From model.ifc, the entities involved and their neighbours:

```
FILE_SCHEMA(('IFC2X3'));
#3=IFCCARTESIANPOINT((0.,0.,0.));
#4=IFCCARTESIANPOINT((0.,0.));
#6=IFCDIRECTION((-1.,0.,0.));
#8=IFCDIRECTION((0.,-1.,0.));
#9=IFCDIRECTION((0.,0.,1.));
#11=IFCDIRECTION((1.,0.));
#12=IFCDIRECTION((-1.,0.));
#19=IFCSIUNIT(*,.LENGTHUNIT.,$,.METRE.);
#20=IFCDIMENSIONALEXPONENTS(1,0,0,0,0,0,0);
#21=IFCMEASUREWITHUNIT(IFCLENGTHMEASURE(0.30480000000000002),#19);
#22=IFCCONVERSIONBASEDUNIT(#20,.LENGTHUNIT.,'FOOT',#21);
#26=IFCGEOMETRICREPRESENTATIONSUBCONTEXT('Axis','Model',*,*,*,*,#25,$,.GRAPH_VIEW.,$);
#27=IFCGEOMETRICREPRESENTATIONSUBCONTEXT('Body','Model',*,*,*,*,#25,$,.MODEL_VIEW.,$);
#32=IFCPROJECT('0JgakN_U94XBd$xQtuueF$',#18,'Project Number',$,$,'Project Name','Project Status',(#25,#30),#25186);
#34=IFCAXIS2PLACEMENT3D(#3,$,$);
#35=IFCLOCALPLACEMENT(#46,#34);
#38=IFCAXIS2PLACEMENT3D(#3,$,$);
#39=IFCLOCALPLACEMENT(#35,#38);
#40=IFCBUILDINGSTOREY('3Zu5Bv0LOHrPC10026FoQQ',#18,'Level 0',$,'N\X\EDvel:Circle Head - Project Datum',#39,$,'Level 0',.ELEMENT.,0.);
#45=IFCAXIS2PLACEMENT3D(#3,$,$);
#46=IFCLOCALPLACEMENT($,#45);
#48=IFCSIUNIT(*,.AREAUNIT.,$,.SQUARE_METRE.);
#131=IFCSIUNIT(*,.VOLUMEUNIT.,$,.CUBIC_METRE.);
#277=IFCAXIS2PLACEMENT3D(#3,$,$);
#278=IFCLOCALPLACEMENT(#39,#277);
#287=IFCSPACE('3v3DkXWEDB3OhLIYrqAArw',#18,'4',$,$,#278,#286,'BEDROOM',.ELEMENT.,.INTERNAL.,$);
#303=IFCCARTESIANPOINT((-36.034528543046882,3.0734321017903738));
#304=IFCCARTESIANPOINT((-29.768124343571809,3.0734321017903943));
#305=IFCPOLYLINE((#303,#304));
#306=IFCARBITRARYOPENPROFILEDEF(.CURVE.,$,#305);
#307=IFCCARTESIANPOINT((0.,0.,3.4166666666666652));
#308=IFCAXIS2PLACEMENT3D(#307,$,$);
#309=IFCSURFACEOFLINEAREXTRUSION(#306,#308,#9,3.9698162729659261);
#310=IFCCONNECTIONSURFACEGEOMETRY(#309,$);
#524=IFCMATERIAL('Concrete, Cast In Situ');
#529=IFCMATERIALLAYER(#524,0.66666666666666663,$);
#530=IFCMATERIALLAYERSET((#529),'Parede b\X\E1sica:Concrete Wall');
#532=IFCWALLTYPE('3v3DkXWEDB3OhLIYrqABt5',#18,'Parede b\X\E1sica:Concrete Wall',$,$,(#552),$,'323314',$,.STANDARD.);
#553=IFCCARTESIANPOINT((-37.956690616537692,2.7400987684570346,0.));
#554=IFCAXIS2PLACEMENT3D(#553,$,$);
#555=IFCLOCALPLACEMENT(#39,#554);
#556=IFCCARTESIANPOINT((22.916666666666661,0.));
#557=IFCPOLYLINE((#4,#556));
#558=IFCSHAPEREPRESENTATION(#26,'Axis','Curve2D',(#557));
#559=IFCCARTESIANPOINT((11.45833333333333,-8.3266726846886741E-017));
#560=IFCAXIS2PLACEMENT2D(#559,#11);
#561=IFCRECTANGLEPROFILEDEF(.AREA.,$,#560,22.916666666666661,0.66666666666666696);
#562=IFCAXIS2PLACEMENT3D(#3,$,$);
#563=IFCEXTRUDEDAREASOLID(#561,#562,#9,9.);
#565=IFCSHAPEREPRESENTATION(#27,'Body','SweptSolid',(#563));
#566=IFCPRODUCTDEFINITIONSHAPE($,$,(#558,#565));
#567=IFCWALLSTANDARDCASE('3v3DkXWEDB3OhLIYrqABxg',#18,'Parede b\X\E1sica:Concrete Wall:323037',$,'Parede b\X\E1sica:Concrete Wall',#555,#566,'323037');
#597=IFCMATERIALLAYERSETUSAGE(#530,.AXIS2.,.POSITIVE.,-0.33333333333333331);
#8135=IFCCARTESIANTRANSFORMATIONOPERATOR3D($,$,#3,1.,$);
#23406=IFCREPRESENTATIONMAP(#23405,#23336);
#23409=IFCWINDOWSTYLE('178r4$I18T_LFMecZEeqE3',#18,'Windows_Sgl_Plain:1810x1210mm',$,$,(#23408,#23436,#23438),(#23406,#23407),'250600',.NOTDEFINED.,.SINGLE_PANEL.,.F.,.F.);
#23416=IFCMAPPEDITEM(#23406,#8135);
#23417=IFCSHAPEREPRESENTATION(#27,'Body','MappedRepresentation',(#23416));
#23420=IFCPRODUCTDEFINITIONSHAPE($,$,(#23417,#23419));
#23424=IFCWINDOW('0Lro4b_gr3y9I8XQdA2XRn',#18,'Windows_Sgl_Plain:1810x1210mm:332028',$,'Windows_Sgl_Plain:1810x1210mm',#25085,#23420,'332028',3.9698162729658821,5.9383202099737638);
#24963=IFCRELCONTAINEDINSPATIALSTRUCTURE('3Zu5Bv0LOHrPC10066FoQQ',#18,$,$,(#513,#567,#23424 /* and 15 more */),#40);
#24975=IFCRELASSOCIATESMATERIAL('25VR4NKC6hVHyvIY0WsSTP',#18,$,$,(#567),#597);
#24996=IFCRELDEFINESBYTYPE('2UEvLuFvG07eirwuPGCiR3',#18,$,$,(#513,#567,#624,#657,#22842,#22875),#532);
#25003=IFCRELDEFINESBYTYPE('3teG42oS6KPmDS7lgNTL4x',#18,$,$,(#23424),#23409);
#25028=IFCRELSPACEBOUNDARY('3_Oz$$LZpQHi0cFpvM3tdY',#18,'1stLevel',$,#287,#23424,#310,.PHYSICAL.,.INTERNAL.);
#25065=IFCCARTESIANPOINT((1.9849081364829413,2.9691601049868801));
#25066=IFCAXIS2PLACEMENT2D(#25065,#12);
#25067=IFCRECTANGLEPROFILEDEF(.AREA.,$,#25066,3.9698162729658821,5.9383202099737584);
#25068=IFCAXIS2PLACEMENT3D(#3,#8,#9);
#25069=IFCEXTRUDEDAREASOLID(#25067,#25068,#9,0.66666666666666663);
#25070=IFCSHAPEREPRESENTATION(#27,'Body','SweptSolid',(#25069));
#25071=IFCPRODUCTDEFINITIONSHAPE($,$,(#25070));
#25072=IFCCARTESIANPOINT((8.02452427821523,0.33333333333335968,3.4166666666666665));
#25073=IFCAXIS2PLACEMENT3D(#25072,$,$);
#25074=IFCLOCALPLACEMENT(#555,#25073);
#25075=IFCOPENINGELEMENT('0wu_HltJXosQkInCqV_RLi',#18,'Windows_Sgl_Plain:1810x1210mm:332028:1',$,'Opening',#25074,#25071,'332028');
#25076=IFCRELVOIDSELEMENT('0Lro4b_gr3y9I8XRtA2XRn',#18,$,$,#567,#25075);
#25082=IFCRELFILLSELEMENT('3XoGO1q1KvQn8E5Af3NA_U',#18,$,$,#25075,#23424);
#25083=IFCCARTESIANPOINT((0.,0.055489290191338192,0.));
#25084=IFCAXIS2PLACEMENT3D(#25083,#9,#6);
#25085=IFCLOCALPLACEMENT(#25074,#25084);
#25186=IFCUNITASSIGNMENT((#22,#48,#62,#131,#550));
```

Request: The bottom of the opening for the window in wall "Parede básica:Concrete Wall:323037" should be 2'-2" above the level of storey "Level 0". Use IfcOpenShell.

```python
import numpy as np
import ifcopenshell
import ifcopenshell.api.geometry
import ifcopenshell.geom
import ifcopenshell.util.element
import ifcopenshell.util.placement
import ifcopenshell.util.shape
import ifcopenshell.util.unit

model = ifcopenshell.open("model.ifc")
unit_scale = ifcopenshell.util.unit.calculate_unit_scale(model)

window = model.by_guid("0Lro4b_gr3y9I8XQdA2XRn")
opening = window.FillsVoids[0].RelatingOpeningElement
storey = ifcopenshell.util.element.get_container(window, ifc_class="IfcBuildingStorey")
level = ifcopenshell.util.placement.get_local_placement(storey.ObjectPlacement)[2, 3]

# The opening's origin need not be at the sill, so measure its lowest point.
shape = ifcopenshell.geom.create_shape(ifcopenshell.geom.settings(), opening)
bottom = ifcopenshell.util.shape.get_shape_bottom_elevation(shape, shape.geometry) / unit_scale
dz = level + 26 * 0.0254 / unit_scale - bottom

shift = np.array([0.0, 0.0, dz])
# The window is placed relative to its opening, so it follows when the opening moves.
matrix = ifcopenshell.util.placement.get_local_placement(opening.ObjectPlacement)
matrix[:3, 3] += shift
ifcopenshell.api.geometry.edit_object_placement(
    model, product=opening, matrix=matrix, is_si=False, should_transform_children=True
)

# Space boundary surfaces are stored in each space's coordinates; move them too.
for rel in window.ProvidesBoundaries:
    if not rel.ConnectionGeometry:
        continue
    surface = rel.ConnectionGeometry.SurfaceOnRelatingElement
    space_matrix = ifcopenshell.util.placement.get_local_placement(rel.RelatingSpace.ObjectPlacement)
    point = np.array(surface.Position.Location.Coordinates) + space_matrix[:3, :3].T @ shift
    surface.Position = model.createIfcAxis2Placement3D(
        model.createIfcCartesianPoint(point.tolist()), surface.Position.Axis, surface.Position.RefDirection
    )

print(f"moved by {dz * unit_scale:+.3f} m")

model.write("model_edited.ifc")
```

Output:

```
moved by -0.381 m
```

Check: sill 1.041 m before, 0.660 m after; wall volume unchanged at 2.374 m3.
